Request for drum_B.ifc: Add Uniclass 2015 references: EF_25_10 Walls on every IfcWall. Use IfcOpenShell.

First a look at what the model holds.

```python
import ifcopenshell

model = ifcopenshell.open("drum_B.ifc")
print(model.schema)
print("classifications:", [c.Name for c in model.by_type("IfcClassification")])
for ifc_class in ("IfcDoor", "IfcRoof", "IfcStair", "IfcWall", "IfcWindow"):
    print(ifc_class, len(model.by_type(ifc_class)))
```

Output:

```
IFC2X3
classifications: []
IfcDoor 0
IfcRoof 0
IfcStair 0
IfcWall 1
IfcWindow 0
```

```python
import ifcopenshell
import ifcopenshell.api.classification

model = ifcopenshell.open("drum_B.ifc")

# IFC2X3 requires Source and Edition and has no link from the project to the system.
system = model.create_entity("IfcClassification", Source="NBS", Edition="2015", Name="Uniclass 2015")

codes = {
    "IfcWall": ("EF_25_10", "Walls"),
}
for ifc_class, (code, name) in codes.items():
    products = model.by_type(ifc_class)
    ifcopenshell.api.classification.add_reference(
        model, products=products, classification=system, identification=code, name=name
    )
    print(code, len(products))

model.write("drum_B_v2.ifc")
```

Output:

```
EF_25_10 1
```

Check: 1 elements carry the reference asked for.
